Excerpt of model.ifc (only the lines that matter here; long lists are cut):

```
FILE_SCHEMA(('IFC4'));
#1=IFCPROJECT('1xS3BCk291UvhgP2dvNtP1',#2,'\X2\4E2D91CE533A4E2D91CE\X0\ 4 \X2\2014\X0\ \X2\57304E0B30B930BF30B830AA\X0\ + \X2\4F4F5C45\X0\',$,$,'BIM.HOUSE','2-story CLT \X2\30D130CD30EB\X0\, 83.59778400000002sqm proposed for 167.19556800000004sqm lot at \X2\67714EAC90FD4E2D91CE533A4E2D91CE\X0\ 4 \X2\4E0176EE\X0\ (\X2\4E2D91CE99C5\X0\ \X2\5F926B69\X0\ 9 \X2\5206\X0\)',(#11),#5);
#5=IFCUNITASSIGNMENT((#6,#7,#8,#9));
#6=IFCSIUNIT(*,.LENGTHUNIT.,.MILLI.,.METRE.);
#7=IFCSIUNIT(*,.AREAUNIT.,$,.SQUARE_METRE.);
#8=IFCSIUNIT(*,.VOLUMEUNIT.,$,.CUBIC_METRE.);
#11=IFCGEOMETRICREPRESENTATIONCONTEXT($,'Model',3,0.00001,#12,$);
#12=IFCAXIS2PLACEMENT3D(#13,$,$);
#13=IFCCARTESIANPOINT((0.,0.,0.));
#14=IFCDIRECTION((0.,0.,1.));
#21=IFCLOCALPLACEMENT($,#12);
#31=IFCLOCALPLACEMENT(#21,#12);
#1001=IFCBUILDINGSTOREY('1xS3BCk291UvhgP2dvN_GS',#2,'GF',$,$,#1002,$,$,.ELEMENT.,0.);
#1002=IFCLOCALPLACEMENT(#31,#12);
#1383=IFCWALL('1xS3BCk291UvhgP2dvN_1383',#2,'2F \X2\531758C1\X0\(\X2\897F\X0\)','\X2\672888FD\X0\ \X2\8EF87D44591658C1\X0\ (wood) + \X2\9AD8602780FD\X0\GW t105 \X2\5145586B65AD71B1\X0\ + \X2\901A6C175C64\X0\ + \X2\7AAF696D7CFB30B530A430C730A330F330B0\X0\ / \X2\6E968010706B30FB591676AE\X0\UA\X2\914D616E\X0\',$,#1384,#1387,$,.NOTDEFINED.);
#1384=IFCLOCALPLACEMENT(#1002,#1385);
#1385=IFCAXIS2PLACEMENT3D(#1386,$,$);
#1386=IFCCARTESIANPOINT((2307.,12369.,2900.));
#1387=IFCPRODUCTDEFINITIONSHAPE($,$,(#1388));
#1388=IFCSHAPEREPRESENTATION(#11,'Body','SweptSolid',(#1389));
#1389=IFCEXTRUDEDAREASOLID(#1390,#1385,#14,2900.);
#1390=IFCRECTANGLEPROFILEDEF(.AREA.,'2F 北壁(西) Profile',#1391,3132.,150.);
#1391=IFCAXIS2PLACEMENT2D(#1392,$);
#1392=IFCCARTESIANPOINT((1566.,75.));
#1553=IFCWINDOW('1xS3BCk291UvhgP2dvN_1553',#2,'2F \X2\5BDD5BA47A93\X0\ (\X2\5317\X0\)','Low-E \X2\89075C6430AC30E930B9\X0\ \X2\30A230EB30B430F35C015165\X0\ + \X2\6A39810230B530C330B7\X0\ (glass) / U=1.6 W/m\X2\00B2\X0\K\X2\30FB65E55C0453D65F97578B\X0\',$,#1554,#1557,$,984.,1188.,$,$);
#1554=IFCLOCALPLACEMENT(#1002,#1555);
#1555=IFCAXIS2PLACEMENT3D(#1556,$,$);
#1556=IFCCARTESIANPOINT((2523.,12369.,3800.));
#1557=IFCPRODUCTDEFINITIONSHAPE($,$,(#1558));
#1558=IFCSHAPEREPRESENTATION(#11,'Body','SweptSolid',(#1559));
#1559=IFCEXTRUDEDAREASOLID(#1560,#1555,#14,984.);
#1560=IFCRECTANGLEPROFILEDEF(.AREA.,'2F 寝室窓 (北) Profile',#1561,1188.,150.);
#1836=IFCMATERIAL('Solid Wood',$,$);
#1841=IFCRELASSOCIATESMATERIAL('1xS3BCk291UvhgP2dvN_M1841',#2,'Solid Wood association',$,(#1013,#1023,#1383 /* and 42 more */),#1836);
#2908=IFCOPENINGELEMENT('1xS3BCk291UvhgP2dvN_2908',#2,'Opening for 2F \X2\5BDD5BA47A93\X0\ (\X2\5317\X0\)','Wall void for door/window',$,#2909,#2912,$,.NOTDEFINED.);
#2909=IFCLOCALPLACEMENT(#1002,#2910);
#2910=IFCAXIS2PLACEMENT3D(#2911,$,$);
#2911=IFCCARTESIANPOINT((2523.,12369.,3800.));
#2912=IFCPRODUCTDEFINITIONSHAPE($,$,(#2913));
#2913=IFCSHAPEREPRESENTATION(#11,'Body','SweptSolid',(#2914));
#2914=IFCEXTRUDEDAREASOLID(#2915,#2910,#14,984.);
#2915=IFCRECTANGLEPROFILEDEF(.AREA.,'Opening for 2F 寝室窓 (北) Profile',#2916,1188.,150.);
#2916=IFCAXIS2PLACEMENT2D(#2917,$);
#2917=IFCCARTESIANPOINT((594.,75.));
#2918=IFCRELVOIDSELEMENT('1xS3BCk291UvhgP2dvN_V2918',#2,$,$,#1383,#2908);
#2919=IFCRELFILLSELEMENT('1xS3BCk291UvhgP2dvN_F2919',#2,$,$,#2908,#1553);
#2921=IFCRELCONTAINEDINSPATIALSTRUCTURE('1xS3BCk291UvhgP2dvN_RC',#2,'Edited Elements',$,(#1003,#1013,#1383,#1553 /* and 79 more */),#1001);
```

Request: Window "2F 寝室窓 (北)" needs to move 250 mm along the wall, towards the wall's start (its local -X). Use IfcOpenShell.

```python
import ifcopenshell
import ifcopenshell.api.geometry
import ifcopenshell.util.placement
import ifcopenshell.util.unit

model = ifcopenshell.open("model.ifc")
unit_scale = ifcopenshell.util.unit.calculate_unit_scale(model)

window = model.by_guid("1xS3BCk291UvhgP2dvN_1553")
opening = window.FillsVoids[0].RelatingOpeningElement
wall = opening.VoidsElements[0].RelatingBuildingElement

wall_matrix = ifcopenshell.util.placement.get_local_placement(wall.ObjectPlacement)
shift = wall_matrix[:3, 0] * -0.25 / unit_scale
before = ifcopenshell.util.placement.get_local_placement(window.ObjectPlacement)[:3, 3].copy()

# The window is not placed relative to its opening, so move both.
for product in (opening, window):
    matrix = ifcopenshell.util.placement.get_local_placement(product.ObjectPlacement)
    matrix[:3, 3] += shift
    ifcopenshell.api.geometry.edit_object_placement(model, product=product, matrix=matrix, is_si=False)

after = ifcopenshell.util.placement.get_local_placement(window.ObjectPlacement)[:3, 3]
print("window moved by", (after - before).round(3) + 0.0)

model.write("model_v2.ifc")
```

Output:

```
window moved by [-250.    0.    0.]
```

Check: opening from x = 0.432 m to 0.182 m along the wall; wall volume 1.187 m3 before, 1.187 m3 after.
